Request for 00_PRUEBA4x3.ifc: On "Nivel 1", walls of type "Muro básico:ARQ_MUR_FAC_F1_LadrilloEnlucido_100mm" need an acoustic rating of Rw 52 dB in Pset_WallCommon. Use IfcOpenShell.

First a look at what the model holds.

```python
import ifcopenshell
import ifcopenshell.util.element

model = ifcopenshell.open("00_PRUEBA4x3.ifc")
print(model.schema)
storey = next(s for s in model.by_type("IfcBuildingStorey") if s.Name == "Nivel 1")
walls = [e for e in ifcopenshell.util.element.get_decomposition(storey) if e.is_a("IfcWall")]
seen = {}
for e in walls:
    element_type = ifcopenshell.util.element.get_type(e)
    key = (element_type.Name if element_type != e and element_type else None, ifcopenshell.util.element.get_pset(e, "Pset_WallCommon", "AcousticRating"))
    seen[key] = seen.get(key, 0) + 1
for (name, value), count in sorted(seen.items(), key=str):
    print(count, "x", name, "|", value)
```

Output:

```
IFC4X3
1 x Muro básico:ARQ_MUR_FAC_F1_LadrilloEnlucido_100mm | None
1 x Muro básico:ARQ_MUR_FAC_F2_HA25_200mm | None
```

```python
import ifcopenshell
import ifcopenshell.api.pset
import ifcopenshell.util.element

model = ifcopenshell.open("00_PRUEBA4x3.ifc")

storey = next(s for s in model.by_type("IfcBuildingStorey") if s.Name == "Nivel 1")
walls = [e for e in ifcopenshell.util.element.get_decomposition(storey) if e.is_a("IfcWall")]

count = 0
for e in walls:
    element_type = ifcopenshell.util.element.get_type(e)
    if element_type in (None, e) or element_type.Name != "Muro básico:ARQ_MUR_FAC_F1_LadrilloEnlucido_100mm":
        continue
    # add_pset returns the element's existing set when there is one.
    pset = ifcopenshell.api.pset.add_pset(model, product=e, name="Pset_WallCommon")
    ifcopenshell.api.pset.edit_pset(model, pset=pset, properties={"AcousticRating": "Rw 52 dB"})
    count += 1

print(count, "walls updated")

model.write("00_PRUEBA4x3_updated.ifc")
```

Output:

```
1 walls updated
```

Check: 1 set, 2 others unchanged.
